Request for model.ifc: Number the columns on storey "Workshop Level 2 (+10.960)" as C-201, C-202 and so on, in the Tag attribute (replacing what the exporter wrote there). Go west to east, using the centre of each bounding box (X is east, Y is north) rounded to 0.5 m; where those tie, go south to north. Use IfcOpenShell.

First a look at what the model holds.

```python
import ifcopenshell
import ifcopenshell.util.element
import ifcopenshell.util.placement

model = ifcopenshell.open("model.ifc")
print(model.schema)
storey = next(s for s in model.by_type("IfcBuildingStorey") if s.Name == "Workshop Level 2 (+10.960)")
columns = [e for e in ifcopenshell.util.element.get_decomposition(storey) if e.is_a("IfcColumn")]
for e in sorted(columns, key=lambda e: e.id()):
    origin = ifcopenshell.util.placement.get_local_placement(e.ObjectPlacement)[:3, 3]
    print(e.id(), e.Tag, e.Name, origin.round(2) + 0.0, sep=" | ")
```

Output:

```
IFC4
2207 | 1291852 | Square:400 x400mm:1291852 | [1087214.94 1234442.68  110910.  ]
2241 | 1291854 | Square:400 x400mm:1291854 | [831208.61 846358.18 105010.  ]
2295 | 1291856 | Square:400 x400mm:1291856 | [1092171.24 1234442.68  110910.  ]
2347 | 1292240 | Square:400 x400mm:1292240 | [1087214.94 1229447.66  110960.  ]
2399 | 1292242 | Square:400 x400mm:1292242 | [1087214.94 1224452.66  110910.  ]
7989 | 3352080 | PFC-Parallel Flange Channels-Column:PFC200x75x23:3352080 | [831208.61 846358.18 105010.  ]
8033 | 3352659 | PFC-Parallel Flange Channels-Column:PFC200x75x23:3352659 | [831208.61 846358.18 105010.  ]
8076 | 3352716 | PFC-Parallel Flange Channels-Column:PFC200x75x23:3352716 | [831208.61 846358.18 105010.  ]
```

```python
import ifcopenshell
import ifcopenshell.geom
import ifcopenshell.util.element
import ifcopenshell.util.shape

model = ifcopenshell.open("model.ifc")
settings = ifcopenshell.geom.settings()
settings.set("use-world-coords", True)


def centre(element):
    shape = ifcopenshell.geom.create_shape(settings, element)
    return ifcopenshell.util.shape.get_bbox_centroid(shape.geometry)


storey = next(s for s in model.by_type("IfcBuildingStorey") if s.Name == "Workshop Level 2 (+10.960)")
columns = [e for e in ifcopenshell.util.element.get_decomposition(storey) if e.is_a("IfcColumn")]

# Insertion points can sit at a corner or the storey origin, so sort by the geometry (in metres).
centres = {e: centre(e) for e in columns}
columns.sort(key=lambda e: (round(centres[e][0] / 0.5), centres[e][1]))

for i, e in enumerate(columns, start=1):
    number = f"C-2{i:02d}"
    e.Tag = number
    print(e.id(), number)

model.write("model_rev.ifc")
```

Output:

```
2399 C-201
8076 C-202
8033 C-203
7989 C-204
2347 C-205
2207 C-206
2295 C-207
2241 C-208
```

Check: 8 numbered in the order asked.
